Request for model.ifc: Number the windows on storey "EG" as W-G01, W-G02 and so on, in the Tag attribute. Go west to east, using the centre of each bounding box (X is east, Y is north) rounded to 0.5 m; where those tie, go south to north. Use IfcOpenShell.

First a look at what the model holds.

```python
import ifcopenshell
import ifcopenshell.util.element
import ifcopenshell.util.placement

model = ifcopenshell.open("model.ifc")
print(model.schema)
storey = next(s for s in model.by_type("IfcBuildingStorey") if s.Name == "EG")
windows = [e for e in ifcopenshell.util.element.get_decomposition(storey) if e.is_a("IfcWindow")]
for e in sorted(windows, key=lambda e: e.id()):
    origin = ifcopenshell.util.placement.get_local_placement(e.ObjectPlacement)[:3, 3]
    print(e.id(), e.Tag, e.Name, origin.round(2) + 0.0, sep=" | ")
```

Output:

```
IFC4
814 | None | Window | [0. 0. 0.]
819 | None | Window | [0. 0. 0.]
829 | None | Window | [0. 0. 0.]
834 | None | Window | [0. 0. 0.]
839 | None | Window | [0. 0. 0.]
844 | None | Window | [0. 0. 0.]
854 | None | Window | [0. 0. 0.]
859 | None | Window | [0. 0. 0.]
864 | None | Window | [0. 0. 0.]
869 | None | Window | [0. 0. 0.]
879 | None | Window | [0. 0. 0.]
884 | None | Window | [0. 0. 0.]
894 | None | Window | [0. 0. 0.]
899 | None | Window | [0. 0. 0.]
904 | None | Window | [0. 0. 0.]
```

```python
import ifcopenshell
import ifcopenshell.geom
import ifcopenshell.util.element
import ifcopenshell.util.shape

model = ifcopenshell.open("model.ifc")
settings = ifcopenshell.geom.settings()
settings.set("use-world-coords", True)


def centre(element):
    shape = ifcopenshell.geom.create_shape(settings, element)
    return ifcopenshell.util.shape.get_bbox_centroid(shape.geometry)


storey = next(s for s in model.by_type("IfcBuildingStorey") if s.Name == "EG")
windows = [e for e in ifcopenshell.util.element.get_decomposition(storey) if e.is_a("IfcWindow")]

# Insertion points can sit at a corner or the storey origin, so sort by the geometry (in metres).
centres = {e: centre(e) for e in windows}
windows.sort(key=lambda e: (round(centres[e][0] / 0.5), centres[e][1]))

for i, e in enumerate(windows, start=1):
    number = f"W-G{i:02d}"
    e.Tag = number
    print(e.id(), number)

model.write("model_v2.ifc")
```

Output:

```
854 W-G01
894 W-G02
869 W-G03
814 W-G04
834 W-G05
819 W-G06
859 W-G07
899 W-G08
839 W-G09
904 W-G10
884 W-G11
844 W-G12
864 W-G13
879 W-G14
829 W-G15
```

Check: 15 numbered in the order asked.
